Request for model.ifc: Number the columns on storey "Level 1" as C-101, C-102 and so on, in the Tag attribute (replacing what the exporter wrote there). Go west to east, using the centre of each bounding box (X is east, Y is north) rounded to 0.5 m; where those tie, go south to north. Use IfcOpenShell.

First a look at what the model holds.

```python
import ifcopenshell
import ifcopenshell.util.element
import ifcopenshell.util.placement

model = ifcopenshell.open("model.ifc")
print(model.schema)
storey = next(s for s in model.by_type("IfcBuildingStorey") if s.Name == "Level 1")
columns = [e for e in ifcopenshell.util.element.get_decomposition(storey) if e.is_a("IfcColumn")]
for e in sorted(columns, key=lambda e: e.id()):
    origin = ifcopenshell.util.placement.get_local_placement(e.ObjectPlacement)[:3, 3]
    print(e.id(), e.Tag, e.Name, origin.round(2) + 0.0, sep=" | ")
```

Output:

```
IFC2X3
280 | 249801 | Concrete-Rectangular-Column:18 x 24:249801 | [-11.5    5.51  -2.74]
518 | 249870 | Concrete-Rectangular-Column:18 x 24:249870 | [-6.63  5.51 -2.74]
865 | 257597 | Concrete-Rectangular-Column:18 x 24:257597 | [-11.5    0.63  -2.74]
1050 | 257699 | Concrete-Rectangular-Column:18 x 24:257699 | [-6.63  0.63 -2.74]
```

```python
import ifcopenshell
import ifcopenshell.geom
import ifcopenshell.util.element
import ifcopenshell.util.shape

model = ifcopenshell.open("model.ifc")
settings = ifcopenshell.geom.settings()
settings.set("use-world-coords", True)


def centre(element):
    shape = ifcopenshell.geom.create_shape(settings, element)
    return ifcopenshell.util.shape.get_bbox_centroid(shape.geometry)


storey = next(s for s in model.by_type("IfcBuildingStorey") if s.Name == "Level 1")
columns = [e for e in ifcopenshell.util.element.get_decomposition(storey) if e.is_a("IfcColumn")]

# Insertion points can sit at a corner or the storey origin, so sort by the geometry (in metres).
centres = {e: centre(e) for e in columns}
columns.sort(key=lambda e: (round(centres[e][0] / 0.5), centres[e][1]))

for i, e in enumerate(columns, start=1):
    number = f"C-1{i:02d}"
    e.Tag = number
    print(e.id(), number)

model.write("model_edited.ifc")
```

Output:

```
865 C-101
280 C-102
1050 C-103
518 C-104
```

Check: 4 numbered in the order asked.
